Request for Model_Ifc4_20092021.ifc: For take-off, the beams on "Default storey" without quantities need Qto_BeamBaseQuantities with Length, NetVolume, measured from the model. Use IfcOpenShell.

First a look at what the model holds.

```python
import ifcopenshell
import ifcopenshell.util.element
import ifcopenshell.util.unit

model = ifcopenshell.open("Model_Ifc4_20092021.ifc")
print(model.schema)
for unit_type in ("LENGTHUNIT", "AREAUNIT", "VOLUMEUNIT"):
    print(unit_type, ifcopenshell.util.unit.calculate_unit_scale(model, unit_type))
storey = next(s for s in model.by_type("IfcBuildingStorey") if s.Name == "Default storey")
beams = [e for e in ifcopenshell.util.element.get_decomposition(storey) if e.is_a("IfcBeam")]
for e in sorted(beams, key=lambda e: e.id()):
    print(e.id(), e.is_a(), e.Name, list(ifcopenshell.util.element.get_psets(e, qtos_only=True)), sep=" | ")
```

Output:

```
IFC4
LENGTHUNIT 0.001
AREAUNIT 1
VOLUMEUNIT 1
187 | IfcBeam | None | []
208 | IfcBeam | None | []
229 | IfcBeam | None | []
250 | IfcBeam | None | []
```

```python
import ifcopenshell
import ifcopenshell.api.pset
import ifcopenshell.geom
import ifcopenshell.util.element
import ifcopenshell.util.shape
import ifcopenshell.util.unit

model = ifcopenshell.open("Model_Ifc4_20092021.ifc")
unit_scale = ifcopenshell.util.unit.calculate_unit_scale(model)
volume_scale = ifcopenshell.util.unit.calculate_unit_scale(model, "VOLUMEUNIT")
settings = ifcopenshell.geom.settings()

storey = next(s for s in model.by_type("IfcBuildingStorey") if s.Name == "Default storey")
beams = [e for e in ifcopenshell.util.element.get_decomposition(storey) if e.is_a("IfcBeam")]

for e in sorted(beams, key=lambda e: e.id()):
    if ifcopenshell.util.element.get_psets(e, qtos_only=True, should_inherit=False):
        continue
    # Geometry comes back in metres, in the element's own axes.
    shape = ifcopenshell.geom.create_shape(settings, e)
    values = {
        "Length": ifcopenshell.util.shape.get_max_xyz(shape.geometry) / unit_scale,
        "NetVolume": ifcopenshell.util.shape.get_volume(shape.geometry) / volume_scale,
    }
    qto = ifcopenshell.api.pset.add_qto(model, product=e, name="Qto_BeamBaseQuantities")
    ifcopenshell.api.pset.edit_qto(model, qto=qto, properties=values)
    print(e.id(), {k: round(v, 3) for k, v in values.items()})

model.write("Model_Ifc4_20092021_updated.ifc")
```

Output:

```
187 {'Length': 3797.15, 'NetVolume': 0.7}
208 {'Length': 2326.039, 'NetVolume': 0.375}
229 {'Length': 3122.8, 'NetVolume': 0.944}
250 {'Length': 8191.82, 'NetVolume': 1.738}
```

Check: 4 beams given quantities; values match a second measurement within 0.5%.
